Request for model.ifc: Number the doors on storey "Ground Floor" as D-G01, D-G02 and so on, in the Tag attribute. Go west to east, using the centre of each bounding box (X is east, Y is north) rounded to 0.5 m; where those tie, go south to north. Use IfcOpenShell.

First a look at what the model holds.

```python
import ifcopenshell
import ifcopenshell.util.element
import ifcopenshell.util.placement

model = ifcopenshell.open("model.ifc")
print(model.schema)
storey = next(s for s in model.by_type("IfcBuildingStorey") if s.Name == "Ground Floor")
doors = [e for e in ifcopenshell.util.element.get_decomposition(storey) if e.is_a("IfcDoor")]
for e in sorted(doors, key=lambda e: e.id()):
    origin = ifcopenshell.util.placement.get_local_placement(e.ObjectPlacement)[:3, 3]
    print(e.id(), e.Tag, e.Name, origin.round(2) + 0.0, sep=" | ")
```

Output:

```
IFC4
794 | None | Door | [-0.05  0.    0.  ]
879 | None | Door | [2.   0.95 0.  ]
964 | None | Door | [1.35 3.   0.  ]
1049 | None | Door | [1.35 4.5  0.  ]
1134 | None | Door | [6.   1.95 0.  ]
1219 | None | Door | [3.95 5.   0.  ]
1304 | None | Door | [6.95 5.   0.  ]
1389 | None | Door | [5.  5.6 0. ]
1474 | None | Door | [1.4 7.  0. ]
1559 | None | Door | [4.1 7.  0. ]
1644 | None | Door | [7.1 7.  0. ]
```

```python
import ifcopenshell
import ifcopenshell.geom
import ifcopenshell.util.element
import ifcopenshell.util.shape

model = ifcopenshell.open("model.ifc")
settings = ifcopenshell.geom.settings()
settings.set("use-world-coords", True)


def centre(element):
    shape = ifcopenshell.geom.create_shape(settings, element)
    return ifcopenshell.util.shape.get_bbox_centroid(shape.geometry)


storey = next(s for s in model.by_type("IfcBuildingStorey") if s.Name == "Ground Floor")
doors = [e for e in ifcopenshell.util.element.get_decomposition(storey) if e.is_a("IfcDoor")]

# Insertion points can sit at a corner or the storey origin, so sort by the geometry (in metres).
centres = {e: centre(e) for e in doors}
doors.sort(key=lambda e: (round(centres[e][0] / 0.5), centres[e][1]))

for i, e in enumerate(doors, start=1):
    number = f"D-G{i:02d}"
    e.Tag = number
    print(e.id(), number)

model.write("model_updated.ifc")
```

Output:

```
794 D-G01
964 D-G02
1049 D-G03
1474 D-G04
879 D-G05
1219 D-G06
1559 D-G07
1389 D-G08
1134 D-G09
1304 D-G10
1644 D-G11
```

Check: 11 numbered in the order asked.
